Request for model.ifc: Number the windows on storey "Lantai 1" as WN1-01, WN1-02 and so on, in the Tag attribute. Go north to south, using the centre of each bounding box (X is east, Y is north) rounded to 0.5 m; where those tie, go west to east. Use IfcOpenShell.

First a look at what the model holds.

```python
import ifcopenshell
import ifcopenshell.util.element
import ifcopenshell.util.placement

model = ifcopenshell.open("model.ifc")
print(model.schema)
storey = next(s for s in model.by_type("IfcBuildingStorey") if s.Name == "Lantai 1")
windows = [e for e in ifcopenshell.util.element.get_decomposition(storey) if e.is_a("IfcWindow")]
for e in sorted(windows, key=lambda e: e.id()):
    origin = ifcopenshell.util.placement.get_local_placement(e.ObjectPlacement)[:3, 3]
    print(e.id(), e.Tag, e.Name, origin.round(2) + 0.0, sep=" | ")
```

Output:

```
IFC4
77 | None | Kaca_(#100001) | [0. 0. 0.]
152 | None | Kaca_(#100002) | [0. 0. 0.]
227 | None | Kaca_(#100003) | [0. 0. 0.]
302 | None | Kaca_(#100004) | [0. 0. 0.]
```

```python
import ifcopenshell
import ifcopenshell.geom
import ifcopenshell.util.element
import ifcopenshell.util.shape

model = ifcopenshell.open("model.ifc")
settings = ifcopenshell.geom.settings()
settings.set("use-world-coords", True)


def centre(element):
    shape = ifcopenshell.geom.create_shape(settings, element)
    return ifcopenshell.util.shape.get_bbox_centroid(shape.geometry)


storey = next(s for s in model.by_type("IfcBuildingStorey") if s.Name == "Lantai 1")
windows = [e for e in ifcopenshell.util.element.get_decomposition(storey) if e.is_a("IfcWindow")]

# Insertion points can sit at a corner or the storey origin, so sort by the geometry (in metres).
centres = {e: centre(e) for e in windows}
windows.sort(key=lambda e: (-round(centres[e][1] / 0.5), centres[e][0]))

for i, e in enumerate(windows, start=1):
    number = f"WN1-{i:02d}"
    e.Tag = number
    print(e.id(), number)

model.write("model-out.ifc")
```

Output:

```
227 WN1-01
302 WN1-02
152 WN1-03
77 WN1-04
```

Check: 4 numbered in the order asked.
